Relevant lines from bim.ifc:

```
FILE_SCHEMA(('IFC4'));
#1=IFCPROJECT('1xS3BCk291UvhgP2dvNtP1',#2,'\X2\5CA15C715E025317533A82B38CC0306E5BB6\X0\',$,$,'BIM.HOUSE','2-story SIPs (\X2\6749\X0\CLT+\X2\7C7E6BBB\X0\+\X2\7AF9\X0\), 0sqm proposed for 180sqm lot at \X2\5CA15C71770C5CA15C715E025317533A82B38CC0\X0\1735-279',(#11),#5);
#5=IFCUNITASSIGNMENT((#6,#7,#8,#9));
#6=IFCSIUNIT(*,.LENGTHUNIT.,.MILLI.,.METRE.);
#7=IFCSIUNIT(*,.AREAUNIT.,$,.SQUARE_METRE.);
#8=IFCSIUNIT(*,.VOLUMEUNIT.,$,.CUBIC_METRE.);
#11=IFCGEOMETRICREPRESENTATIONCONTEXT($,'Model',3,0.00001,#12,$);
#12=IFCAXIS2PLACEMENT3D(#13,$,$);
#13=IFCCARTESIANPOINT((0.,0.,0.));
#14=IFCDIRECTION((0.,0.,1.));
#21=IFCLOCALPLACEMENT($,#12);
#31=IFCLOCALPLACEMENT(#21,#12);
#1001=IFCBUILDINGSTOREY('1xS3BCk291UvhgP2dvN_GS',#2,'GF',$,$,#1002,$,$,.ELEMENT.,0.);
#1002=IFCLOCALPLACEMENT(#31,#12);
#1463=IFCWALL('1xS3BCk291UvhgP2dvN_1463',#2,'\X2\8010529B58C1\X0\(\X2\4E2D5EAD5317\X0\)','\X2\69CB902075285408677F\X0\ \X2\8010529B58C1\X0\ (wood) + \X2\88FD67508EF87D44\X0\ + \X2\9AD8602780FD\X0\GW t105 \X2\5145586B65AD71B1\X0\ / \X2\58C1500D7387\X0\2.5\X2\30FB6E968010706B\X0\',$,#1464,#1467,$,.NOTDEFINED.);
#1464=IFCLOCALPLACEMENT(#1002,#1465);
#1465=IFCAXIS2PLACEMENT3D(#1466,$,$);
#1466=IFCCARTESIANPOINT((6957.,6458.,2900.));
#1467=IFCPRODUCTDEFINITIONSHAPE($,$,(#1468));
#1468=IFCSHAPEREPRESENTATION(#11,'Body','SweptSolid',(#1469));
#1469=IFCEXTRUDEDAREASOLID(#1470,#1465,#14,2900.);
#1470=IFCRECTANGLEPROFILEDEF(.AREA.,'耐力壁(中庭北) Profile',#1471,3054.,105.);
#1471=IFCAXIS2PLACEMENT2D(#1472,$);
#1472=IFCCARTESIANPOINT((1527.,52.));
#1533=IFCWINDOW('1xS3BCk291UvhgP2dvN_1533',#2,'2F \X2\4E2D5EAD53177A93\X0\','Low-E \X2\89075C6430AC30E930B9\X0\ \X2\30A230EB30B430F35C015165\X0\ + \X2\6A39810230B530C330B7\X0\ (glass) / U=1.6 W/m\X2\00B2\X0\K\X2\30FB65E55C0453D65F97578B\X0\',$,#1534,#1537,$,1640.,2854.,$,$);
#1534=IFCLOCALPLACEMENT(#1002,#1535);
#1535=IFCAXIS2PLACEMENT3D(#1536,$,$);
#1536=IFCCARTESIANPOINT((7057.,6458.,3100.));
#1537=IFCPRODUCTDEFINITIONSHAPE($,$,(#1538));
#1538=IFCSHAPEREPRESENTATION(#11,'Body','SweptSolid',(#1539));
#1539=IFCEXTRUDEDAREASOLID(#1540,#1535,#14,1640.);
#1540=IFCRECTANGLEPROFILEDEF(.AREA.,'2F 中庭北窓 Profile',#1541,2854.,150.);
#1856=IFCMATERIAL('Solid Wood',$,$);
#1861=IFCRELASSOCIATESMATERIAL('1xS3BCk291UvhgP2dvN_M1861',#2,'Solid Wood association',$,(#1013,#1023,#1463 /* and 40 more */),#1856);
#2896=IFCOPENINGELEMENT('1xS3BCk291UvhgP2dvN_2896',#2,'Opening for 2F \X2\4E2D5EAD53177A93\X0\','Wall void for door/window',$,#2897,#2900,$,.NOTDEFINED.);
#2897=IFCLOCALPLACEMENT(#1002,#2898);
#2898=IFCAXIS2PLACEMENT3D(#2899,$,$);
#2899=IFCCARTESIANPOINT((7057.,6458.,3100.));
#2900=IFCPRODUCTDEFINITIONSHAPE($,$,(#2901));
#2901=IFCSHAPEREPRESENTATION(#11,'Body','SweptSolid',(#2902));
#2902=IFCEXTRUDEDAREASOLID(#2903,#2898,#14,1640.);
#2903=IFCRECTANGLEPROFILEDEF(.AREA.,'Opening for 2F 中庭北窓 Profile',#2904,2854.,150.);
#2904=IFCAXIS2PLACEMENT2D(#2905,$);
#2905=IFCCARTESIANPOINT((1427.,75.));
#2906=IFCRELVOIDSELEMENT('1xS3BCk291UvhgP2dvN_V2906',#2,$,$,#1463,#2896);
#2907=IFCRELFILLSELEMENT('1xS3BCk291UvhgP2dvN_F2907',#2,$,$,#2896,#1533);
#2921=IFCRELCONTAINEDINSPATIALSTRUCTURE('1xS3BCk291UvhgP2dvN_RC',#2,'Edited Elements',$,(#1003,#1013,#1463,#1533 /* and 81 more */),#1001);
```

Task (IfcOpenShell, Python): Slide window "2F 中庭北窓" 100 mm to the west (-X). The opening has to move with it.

```python
import ifcopenshell
import ifcopenshell.api.geometry
import ifcopenshell.util.placement
import ifcopenshell.util.unit

model = ifcopenshell.open("bim.ifc")
unit_scale = ifcopenshell.util.unit.calculate_unit_scale(model)

window = model.by_id(1533)
opening = window.FillsVoids[0].RelatingOpeningElement
wall = opening.VoidsElements[0].RelatingBuildingElement

wall_matrix = ifcopenshell.util.placement.get_local_placement(wall.ObjectPlacement)
shift = wall_matrix[:3, 0] * -0.1 / unit_scale
before = ifcopenshell.util.placement.get_local_placement(window.ObjectPlacement)[:3, 3].copy()

# The window is not placed relative to its opening, so move both.
for product in (opening, window):
    matrix = ifcopenshell.util.placement.get_local_placement(product.ObjectPlacement)
    matrix[:3, 3] += shift
    ifcopenshell.api.geometry.edit_object_placement(model, product=product, matrix=matrix, is_si=False)

after = ifcopenshell.util.placement.get_local_placement(window.ObjectPlacement)[:3, 3]
print("window moved by", (after - before).round(3) + 0.0)

model.write("bim_v2.ifc")
```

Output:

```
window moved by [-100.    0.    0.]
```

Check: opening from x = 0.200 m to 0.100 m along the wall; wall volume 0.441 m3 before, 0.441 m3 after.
